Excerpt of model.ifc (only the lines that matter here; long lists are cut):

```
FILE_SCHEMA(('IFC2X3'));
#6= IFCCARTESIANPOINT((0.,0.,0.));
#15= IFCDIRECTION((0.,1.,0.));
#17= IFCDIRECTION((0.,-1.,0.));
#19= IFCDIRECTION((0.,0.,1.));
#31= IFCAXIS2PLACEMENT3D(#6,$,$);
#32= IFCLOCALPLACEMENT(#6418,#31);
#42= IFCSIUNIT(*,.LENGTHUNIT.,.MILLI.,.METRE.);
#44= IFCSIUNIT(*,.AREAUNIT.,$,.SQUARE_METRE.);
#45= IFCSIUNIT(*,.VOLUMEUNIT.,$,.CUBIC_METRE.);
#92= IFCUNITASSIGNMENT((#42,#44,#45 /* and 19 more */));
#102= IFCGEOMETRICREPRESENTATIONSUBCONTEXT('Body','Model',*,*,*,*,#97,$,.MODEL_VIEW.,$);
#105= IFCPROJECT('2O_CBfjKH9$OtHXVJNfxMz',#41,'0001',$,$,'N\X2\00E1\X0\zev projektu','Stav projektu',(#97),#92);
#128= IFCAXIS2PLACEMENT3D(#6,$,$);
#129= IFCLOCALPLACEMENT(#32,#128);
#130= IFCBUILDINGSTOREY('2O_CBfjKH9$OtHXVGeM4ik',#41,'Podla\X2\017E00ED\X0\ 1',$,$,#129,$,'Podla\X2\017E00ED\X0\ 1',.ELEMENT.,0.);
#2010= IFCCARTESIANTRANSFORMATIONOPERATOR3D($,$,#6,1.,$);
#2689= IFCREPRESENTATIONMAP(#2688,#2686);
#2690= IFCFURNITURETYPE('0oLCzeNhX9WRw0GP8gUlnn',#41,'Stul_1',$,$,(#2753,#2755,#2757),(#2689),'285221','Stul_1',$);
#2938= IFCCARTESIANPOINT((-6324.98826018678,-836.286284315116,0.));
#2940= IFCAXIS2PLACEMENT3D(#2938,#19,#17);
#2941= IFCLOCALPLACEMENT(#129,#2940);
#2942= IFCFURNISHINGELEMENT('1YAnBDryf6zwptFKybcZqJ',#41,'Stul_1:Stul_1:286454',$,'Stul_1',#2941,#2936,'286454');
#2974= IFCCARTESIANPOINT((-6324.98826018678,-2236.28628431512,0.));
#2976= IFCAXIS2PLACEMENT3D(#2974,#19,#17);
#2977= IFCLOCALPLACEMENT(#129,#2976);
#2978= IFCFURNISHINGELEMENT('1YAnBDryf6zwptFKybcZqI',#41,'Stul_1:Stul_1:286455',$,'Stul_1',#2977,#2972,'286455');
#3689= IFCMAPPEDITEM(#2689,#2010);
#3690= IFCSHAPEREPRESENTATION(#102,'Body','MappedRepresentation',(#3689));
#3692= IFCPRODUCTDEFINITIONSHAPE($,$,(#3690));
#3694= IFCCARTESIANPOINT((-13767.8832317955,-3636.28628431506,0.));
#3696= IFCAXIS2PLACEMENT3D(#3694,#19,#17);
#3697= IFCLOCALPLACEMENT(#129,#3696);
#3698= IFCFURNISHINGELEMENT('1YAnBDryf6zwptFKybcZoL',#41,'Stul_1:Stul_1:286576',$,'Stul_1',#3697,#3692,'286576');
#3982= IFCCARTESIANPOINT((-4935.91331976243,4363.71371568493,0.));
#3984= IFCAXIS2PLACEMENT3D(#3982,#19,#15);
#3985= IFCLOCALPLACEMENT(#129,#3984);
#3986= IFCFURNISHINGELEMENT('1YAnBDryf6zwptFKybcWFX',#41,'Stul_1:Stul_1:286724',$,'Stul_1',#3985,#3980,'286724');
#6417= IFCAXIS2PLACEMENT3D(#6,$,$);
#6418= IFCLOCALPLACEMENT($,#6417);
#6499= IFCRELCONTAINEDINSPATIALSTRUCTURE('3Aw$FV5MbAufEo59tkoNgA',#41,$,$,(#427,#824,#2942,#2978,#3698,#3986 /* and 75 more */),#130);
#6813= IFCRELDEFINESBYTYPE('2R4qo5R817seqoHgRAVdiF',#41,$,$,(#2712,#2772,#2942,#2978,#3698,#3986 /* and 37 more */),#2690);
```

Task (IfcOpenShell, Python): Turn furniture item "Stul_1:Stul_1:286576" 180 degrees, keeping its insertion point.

```python
import ifcopenshell
import ifcopenshell.api.geometry
import ifcopenshell.util.placement

model = ifcopenshell.open("model.ifc")

item = model.by_id(3698)
matrix = ifcopenshell.util.placement.get_local_placement(item.ObjectPlacement)
matrix = matrix @ ifcopenshell.util.placement.rotation(180, "Z")
ifcopenshell.api.geometry.edit_object_placement(model, product=item, matrix=matrix, is_si=False)

print(ifcopenshell.util.placement.get_local_placement(item.ObjectPlacement).round(3) + 0.0)

model.write("model_updated.ifc")
```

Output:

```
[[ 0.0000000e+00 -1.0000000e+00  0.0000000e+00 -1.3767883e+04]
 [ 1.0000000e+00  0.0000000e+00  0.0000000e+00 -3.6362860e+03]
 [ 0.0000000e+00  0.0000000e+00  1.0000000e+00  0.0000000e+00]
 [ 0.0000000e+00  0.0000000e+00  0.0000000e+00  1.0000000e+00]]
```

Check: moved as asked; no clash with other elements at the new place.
